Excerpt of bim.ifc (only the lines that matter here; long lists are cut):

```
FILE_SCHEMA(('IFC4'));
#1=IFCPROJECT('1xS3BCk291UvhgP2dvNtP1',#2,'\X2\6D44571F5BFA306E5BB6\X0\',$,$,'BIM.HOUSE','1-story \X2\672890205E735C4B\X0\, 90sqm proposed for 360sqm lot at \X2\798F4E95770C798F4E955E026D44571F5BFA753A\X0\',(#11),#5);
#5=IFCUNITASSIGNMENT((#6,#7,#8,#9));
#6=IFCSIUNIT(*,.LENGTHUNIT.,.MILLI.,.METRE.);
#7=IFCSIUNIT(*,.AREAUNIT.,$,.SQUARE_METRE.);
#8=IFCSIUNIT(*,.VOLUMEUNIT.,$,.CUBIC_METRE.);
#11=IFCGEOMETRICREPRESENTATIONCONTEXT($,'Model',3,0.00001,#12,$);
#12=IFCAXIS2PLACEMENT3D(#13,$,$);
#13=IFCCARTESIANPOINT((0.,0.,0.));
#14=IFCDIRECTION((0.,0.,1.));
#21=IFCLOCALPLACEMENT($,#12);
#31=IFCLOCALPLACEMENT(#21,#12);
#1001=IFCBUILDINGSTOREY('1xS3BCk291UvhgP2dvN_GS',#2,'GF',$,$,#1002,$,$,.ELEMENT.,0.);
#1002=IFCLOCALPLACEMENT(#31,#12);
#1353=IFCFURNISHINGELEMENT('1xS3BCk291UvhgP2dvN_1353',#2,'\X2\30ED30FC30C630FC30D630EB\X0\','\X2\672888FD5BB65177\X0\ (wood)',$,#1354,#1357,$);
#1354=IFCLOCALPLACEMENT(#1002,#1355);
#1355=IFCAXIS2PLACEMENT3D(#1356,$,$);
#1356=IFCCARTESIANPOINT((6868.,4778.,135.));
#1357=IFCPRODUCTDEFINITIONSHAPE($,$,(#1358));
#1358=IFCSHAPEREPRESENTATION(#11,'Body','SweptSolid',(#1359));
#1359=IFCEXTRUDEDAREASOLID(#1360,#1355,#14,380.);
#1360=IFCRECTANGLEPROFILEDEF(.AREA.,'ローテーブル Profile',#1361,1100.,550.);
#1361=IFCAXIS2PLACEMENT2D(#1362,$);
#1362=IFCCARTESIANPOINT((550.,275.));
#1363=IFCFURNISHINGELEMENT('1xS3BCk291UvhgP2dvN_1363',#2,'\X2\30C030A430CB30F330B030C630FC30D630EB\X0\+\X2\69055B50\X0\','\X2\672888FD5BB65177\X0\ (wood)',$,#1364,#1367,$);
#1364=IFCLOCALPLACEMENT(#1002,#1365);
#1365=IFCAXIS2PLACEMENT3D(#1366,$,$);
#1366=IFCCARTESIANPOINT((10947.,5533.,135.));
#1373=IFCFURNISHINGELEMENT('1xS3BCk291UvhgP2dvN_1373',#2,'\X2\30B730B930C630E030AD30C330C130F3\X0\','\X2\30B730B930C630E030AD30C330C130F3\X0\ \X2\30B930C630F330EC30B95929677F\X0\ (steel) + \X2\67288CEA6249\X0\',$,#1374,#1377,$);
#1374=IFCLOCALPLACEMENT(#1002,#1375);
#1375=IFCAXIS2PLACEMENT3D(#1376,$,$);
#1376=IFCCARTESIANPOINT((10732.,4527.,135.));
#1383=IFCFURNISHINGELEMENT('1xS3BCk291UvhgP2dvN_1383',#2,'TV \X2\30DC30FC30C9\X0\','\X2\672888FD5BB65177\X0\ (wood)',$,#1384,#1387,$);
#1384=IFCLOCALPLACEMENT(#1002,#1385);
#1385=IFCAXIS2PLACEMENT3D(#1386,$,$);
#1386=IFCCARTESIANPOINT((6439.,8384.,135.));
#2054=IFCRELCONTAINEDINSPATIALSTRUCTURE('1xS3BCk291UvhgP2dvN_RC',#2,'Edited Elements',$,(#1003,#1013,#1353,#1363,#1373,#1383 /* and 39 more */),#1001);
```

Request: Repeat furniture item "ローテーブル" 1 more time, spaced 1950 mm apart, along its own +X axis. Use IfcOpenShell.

```python
import ifcopenshell
import ifcopenshell.api.geometry
import ifcopenshell.api.root
import ifcopenshell.util.element
import ifcopenshell.util.placement

model = ifcopenshell.open("bim.ifc")


def reuse_history(source, copy):
    """copy_class also copies each property set's owner history, people and application; keep the originals."""
    for rel in copy.IsDefinedBy:
        if rel.is_a("IfcRelDefinesByProperties") and (history := rel.RelatingPropertyDefinition.OwnerHistory):
            rel.RelatingPropertyDefinition.OwnerHistory = source.OwnerHistory
            ifcopenshell.util.element.remove_deep2(model, history)


source = model.by_guid("1xS3BCk291UvhgP2dvN_1353")
base = ifcopenshell.util.placement.get_local_placement(source.ObjectPlacement)
step = base[:3, 0] * 1950.0

for i in range(1, 2):
    copy = ifcopenshell.api.root.copy_class(model, product=source)
    copy.Representation = ifcopenshell.util.element.copy_deep(
        model, source.Representation, exclude=["IfcGeometricRepresentationContext", "IfcRepresentationMap"]
    )
    reuse_history(source, copy)
    matrix = base.copy()
    matrix[:3, 3] += i * step
    print("added at", matrix[:3, 3].round(3) + 0.0)
    ifcopenshell.api.geometry.edit_object_placement(model, product=copy, matrix=matrix, is_si=False)

model.write("bim_v2.ifc")
```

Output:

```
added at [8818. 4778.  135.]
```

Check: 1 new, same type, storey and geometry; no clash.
